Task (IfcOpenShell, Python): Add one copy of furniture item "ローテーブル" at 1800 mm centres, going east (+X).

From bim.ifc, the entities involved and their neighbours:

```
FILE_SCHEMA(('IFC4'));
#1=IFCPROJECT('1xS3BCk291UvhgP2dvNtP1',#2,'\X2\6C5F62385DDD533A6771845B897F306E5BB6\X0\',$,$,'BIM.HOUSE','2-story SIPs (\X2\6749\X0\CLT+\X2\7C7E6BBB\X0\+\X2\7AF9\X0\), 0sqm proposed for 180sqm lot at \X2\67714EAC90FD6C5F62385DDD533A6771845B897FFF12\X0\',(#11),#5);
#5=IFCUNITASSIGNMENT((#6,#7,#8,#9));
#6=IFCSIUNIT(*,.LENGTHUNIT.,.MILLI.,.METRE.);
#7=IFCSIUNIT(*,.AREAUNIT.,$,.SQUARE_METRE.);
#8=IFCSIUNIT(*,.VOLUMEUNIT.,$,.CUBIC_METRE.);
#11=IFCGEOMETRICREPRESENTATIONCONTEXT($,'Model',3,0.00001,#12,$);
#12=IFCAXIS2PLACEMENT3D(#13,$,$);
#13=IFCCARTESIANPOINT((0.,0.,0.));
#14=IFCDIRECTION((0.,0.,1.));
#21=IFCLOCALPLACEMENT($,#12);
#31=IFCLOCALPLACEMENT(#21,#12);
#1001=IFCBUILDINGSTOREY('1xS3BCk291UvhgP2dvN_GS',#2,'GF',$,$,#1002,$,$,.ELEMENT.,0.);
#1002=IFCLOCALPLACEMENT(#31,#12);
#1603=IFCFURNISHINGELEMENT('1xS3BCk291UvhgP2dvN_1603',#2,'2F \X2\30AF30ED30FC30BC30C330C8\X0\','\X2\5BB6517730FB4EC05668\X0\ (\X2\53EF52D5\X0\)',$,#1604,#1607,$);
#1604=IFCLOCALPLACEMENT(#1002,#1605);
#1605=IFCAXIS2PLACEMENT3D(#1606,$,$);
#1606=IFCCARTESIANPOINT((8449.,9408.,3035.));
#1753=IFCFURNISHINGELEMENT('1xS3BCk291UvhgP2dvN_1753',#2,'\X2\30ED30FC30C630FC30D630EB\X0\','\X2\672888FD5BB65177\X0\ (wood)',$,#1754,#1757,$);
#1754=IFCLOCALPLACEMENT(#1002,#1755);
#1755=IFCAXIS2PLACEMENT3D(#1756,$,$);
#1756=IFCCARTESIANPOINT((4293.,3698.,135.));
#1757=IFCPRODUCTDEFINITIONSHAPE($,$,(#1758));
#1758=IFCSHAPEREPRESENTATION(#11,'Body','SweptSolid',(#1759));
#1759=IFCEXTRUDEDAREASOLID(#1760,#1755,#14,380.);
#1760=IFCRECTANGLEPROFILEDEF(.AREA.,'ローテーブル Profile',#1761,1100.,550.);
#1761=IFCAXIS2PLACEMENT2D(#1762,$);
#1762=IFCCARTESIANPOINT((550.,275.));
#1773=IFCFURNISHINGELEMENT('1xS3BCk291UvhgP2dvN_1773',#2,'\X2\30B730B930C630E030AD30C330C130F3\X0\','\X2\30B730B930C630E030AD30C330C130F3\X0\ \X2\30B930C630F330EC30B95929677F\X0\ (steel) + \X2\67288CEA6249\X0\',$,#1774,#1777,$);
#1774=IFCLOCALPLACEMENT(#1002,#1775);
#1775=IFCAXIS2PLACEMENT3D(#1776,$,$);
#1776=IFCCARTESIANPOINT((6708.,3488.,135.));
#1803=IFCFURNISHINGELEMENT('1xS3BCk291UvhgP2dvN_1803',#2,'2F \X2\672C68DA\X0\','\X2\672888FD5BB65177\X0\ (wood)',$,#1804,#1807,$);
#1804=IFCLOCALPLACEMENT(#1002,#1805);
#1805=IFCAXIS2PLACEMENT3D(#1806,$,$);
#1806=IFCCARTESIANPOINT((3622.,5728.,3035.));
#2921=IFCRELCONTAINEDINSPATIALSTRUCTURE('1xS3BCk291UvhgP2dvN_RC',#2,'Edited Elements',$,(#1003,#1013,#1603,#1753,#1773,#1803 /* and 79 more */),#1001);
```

```python
import numpy as np
import ifcopenshell
import ifcopenshell.api.geometry
import ifcopenshell.api.root
import ifcopenshell.util.element
import ifcopenshell.util.placement
import ifcopenshell.util.unit

model = ifcopenshell.open("bim.ifc")
unit_scale = ifcopenshell.util.unit.calculate_unit_scale(model)


def reuse_history(source, copy):
    """copy_class also copies each property set's owner history, people and application; keep the originals."""
    for rel in copy.IsDefinedBy:
        if rel.is_a("IfcRelDefinesByProperties") and (history := rel.RelatingPropertyDefinition.OwnerHistory):
            rel.RelatingPropertyDefinition.OwnerHistory = source.OwnerHistory
            ifcopenshell.util.element.remove_deep2(model, history)


source = model.by_guid("1xS3BCk291UvhgP2dvN_1753")
base = ifcopenshell.util.placement.get_local_placement(source.ObjectPlacement)
step = np.array([1.0, 0.0, 0.0]) * 1.8 / unit_scale

for i in range(1, 2):
    copy = ifcopenshell.api.root.copy_class(model, product=source)
    copy.Representation = ifcopenshell.util.element.copy_deep(
        model, source.Representation, exclude=["IfcGeometricRepresentationContext", "IfcRepresentationMap"]
    )
    reuse_history(source, copy)
    matrix = base.copy()
    matrix[:3, 3] += i * step
    print("added at", matrix[:3, 3].round(3) + 0.0)
    ifcopenshell.api.geometry.edit_object_placement(model, product=copy, matrix=matrix, is_si=False)

model.write("bim_edited.ifc")
```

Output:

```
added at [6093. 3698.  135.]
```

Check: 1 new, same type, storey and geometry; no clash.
